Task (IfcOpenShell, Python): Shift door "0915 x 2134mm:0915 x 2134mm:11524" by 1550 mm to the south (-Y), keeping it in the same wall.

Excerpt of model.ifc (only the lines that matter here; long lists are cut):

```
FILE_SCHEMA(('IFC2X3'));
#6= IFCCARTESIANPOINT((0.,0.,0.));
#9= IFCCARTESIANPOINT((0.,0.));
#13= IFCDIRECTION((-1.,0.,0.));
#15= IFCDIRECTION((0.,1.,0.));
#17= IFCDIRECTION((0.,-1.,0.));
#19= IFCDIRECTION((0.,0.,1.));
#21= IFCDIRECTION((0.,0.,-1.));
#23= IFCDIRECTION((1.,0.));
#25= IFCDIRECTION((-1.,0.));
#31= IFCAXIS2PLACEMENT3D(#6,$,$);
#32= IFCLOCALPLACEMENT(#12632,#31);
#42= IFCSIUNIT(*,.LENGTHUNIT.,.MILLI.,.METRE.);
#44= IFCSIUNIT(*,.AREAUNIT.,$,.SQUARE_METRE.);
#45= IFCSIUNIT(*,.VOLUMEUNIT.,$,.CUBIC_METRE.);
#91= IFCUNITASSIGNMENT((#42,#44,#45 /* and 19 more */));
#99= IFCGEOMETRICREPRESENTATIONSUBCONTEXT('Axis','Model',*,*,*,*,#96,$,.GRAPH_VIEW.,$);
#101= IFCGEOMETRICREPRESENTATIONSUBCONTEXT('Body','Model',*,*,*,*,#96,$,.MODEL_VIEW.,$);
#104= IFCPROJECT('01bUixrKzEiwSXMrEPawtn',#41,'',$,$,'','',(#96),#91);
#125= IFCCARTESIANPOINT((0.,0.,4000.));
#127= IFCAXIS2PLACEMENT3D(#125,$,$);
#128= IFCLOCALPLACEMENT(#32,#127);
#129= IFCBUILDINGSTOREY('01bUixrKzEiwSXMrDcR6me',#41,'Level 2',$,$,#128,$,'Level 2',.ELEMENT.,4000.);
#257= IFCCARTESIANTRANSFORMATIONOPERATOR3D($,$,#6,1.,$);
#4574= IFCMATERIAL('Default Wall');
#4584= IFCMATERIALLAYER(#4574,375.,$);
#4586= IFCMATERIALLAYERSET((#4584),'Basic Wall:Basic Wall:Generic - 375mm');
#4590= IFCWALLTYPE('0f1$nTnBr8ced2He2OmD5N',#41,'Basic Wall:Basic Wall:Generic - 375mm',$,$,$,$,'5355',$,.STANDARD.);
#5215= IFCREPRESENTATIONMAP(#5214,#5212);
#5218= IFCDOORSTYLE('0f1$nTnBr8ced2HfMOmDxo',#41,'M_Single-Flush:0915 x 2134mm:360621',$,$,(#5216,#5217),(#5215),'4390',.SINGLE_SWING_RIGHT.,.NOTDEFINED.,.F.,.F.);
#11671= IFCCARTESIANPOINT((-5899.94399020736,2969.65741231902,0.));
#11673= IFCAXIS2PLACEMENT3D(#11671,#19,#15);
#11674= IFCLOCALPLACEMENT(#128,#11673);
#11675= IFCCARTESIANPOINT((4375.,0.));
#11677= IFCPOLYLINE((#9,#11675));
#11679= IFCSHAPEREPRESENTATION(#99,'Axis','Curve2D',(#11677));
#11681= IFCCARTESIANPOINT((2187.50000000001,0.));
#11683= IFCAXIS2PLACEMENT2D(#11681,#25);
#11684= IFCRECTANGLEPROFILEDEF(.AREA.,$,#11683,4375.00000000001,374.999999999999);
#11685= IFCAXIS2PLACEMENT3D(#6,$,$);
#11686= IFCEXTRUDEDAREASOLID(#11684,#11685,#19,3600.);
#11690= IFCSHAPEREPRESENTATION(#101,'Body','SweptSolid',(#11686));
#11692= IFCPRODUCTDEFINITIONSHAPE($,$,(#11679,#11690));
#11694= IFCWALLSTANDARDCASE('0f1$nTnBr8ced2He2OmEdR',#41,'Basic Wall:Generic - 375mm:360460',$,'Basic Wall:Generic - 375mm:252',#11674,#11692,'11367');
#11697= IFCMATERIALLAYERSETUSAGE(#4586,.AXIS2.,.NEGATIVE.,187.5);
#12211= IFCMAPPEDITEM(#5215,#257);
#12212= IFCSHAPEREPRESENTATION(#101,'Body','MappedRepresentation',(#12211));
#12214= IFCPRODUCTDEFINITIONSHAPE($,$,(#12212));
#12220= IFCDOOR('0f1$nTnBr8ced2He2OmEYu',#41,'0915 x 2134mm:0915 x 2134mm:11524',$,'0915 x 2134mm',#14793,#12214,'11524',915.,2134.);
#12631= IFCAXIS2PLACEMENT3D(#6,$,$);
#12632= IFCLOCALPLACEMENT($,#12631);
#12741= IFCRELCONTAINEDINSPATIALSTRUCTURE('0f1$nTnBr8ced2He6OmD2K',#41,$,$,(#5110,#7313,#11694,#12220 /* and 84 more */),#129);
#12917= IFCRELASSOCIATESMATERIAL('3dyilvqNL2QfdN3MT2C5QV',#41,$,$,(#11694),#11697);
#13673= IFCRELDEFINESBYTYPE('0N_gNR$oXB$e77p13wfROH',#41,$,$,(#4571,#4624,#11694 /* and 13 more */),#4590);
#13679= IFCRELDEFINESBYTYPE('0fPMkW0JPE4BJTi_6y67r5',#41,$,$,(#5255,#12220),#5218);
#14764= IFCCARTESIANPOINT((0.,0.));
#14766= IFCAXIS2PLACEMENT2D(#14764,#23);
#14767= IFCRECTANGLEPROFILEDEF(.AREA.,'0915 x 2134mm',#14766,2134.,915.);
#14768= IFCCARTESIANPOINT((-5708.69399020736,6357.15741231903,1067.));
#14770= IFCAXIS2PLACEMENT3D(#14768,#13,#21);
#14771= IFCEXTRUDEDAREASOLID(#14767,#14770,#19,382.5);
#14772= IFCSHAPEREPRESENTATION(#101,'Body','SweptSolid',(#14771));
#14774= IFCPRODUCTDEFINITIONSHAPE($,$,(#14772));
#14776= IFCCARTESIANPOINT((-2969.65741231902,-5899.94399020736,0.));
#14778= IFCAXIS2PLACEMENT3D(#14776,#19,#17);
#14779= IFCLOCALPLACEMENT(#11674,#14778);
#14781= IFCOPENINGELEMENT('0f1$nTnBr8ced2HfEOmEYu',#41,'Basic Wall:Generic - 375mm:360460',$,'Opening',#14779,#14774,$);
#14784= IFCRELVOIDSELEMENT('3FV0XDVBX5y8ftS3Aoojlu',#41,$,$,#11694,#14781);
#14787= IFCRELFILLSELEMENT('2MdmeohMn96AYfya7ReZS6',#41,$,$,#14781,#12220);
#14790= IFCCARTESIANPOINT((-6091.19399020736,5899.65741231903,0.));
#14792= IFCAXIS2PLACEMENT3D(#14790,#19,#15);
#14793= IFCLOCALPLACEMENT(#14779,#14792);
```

```python
import ifcopenshell
import ifcopenshell.api.geometry
import ifcopenshell.util.placement

model = ifcopenshell.open("model.ifc")

door = model.by_guid("0f1$nTnBr8ced2He2OmEYu")
opening = door.FillsVoids[0].RelatingOpeningElement
wall = opening.VoidsElements[0].RelatingBuildingElement

wall_matrix = ifcopenshell.util.placement.get_local_placement(wall.ObjectPlacement)
shift = wall_matrix[:3, 0] * -1550.0
before = ifcopenshell.util.placement.get_local_placement(door.ObjectPlacement)[:3, 3].copy()

# The door is placed relative to its opening, so it follows when the opening moves.
matrix = ifcopenshell.util.placement.get_local_placement(opening.ObjectPlacement)
matrix[:3, 3] += shift
ifcopenshell.api.geometry.edit_object_placement(
    model, product=opening, matrix=matrix, is_si=False, should_transform_children=True
)

after = ifcopenshell.util.placement.get_local_placement(door.ObjectPlacement)[:3, 3]
print("door moved by", (after - before).round(3) + 0.0)

model.write("model_v2.ifc")
```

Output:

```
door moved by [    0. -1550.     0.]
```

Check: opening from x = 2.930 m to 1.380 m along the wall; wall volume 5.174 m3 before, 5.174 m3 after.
